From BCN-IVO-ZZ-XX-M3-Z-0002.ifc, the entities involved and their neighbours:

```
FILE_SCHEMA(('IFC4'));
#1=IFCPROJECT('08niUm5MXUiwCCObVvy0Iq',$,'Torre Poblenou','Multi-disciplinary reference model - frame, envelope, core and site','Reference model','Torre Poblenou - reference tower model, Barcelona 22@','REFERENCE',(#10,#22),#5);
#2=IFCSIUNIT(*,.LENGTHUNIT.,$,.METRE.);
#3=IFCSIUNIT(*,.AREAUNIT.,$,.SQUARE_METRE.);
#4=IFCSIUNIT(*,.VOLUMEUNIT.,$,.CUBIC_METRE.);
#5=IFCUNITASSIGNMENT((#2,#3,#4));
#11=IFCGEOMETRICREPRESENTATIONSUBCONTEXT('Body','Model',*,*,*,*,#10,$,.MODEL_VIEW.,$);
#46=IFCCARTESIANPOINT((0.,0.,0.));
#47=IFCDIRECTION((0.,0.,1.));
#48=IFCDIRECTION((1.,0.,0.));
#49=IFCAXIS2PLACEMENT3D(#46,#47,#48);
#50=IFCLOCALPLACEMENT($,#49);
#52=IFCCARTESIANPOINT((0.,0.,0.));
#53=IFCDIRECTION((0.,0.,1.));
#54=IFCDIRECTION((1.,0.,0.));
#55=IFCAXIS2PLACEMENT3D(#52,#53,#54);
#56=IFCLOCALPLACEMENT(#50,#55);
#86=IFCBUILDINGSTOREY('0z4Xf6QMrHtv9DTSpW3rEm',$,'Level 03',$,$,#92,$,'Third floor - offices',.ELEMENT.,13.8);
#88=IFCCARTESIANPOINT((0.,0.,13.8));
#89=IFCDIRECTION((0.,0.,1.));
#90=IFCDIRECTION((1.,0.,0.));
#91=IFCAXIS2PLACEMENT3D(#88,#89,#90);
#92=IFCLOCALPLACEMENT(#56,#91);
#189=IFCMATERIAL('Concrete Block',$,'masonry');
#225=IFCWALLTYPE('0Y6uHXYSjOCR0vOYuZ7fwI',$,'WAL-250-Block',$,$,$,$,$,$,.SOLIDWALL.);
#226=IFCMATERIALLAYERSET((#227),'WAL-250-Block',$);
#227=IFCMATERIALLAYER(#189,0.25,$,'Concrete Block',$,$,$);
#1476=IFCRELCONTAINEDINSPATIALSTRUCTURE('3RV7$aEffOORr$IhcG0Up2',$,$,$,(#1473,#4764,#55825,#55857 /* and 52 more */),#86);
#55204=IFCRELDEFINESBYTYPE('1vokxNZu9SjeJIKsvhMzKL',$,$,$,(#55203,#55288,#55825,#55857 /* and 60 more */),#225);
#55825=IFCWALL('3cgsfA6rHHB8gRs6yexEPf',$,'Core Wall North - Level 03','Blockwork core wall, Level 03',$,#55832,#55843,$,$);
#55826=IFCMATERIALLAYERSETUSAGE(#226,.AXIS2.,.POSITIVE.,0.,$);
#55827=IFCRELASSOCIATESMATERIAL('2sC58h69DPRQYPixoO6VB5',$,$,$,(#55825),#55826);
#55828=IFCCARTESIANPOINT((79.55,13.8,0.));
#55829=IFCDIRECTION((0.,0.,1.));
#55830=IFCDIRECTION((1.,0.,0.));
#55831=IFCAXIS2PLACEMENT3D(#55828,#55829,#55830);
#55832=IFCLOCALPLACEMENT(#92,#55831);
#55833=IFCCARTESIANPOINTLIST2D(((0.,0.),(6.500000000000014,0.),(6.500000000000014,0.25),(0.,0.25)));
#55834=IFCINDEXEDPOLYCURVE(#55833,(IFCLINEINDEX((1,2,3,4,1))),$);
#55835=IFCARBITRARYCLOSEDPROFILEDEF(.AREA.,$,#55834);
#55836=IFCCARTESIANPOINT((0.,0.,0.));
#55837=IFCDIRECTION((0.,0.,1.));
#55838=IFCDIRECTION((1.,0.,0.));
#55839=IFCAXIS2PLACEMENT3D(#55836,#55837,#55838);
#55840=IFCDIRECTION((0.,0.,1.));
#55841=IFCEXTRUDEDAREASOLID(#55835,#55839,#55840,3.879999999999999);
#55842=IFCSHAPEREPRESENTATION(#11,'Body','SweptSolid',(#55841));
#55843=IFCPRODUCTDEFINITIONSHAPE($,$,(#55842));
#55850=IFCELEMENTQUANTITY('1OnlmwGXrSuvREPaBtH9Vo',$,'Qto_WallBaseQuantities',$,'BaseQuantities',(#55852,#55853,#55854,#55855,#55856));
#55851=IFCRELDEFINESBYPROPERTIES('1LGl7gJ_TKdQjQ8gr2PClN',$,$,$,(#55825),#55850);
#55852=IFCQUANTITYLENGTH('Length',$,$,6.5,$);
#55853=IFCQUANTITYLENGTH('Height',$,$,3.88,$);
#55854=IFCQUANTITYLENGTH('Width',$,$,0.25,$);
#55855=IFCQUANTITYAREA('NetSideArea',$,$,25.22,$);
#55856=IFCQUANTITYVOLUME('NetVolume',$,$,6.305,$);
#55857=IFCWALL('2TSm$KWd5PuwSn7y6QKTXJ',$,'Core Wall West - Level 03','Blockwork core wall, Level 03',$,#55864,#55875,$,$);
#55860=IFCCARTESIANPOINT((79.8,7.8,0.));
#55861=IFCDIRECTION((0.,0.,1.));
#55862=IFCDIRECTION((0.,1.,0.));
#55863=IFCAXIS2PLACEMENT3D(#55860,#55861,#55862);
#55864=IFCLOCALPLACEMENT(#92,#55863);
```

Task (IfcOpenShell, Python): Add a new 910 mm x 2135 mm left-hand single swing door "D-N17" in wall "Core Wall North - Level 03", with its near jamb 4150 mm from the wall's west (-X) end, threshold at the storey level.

```python
import numpy as np
import ifcopenshell
import ifcopenshell.api.feature
import ifcopenshell.api.geometry
import ifcopenshell.api.pset
import ifcopenshell.api.root
import ifcopenshell.api.spatial
import ifcopenshell.geom
import ifcopenshell.util.element
import ifcopenshell.util.placement
import ifcopenshell.util.representation
import ifcopenshell.util.shape
import ifcopenshell.util.unit

model = ifcopenshell.open("BCN-IVO-ZZ-XX-M3-Z-0002.ifc")
unit_scale = ifcopenshell.util.unit.calculate_unit_scale(model)
area_scale = ifcopenshell.util.unit.calculate_unit_scale(model, "AREAUNIT")
volume_scale = ifcopenshell.util.unit.calculate_unit_scale(model, "VOLUMEUNIT")
settings = ifcopenshell.geom.settings()


def volume(element):
    """Net volume in cubic metres, openings subtracted."""
    shape = ifcopenshell.geom.create_shape(settings, element)
    return ifcopenshell.util.shape.get_volume(shape.geometry)


wall = model.by_guid("3cgsfA6rHHB8gRs6yexEPf")
storey = ifcopenshell.util.element.get_container(wall, ifc_class="IfcBuildingStorey")
context = ifcopenshell.util.representation.get_context(model, "Model", "Body", "MODEL_VIEW")
before = volume(wall)

width, height, from_end, sill = 0.91, 2.135, 4.15, 0.0  # metres

# The wall runs along its own X axis, and the end named is its -X end.
wall_shape = ifcopenshell.geom.create_shape(settings, wall)
x, y, z = ifcopenshell.util.shape.get_vertices(wall_shape.geometry).T
start = x.min() + from_end
face, thickness = float(y.min()), float(y.max() - y.min())
wall_matrix = ifcopenshell.util.placement.get_local_placement(wall.ObjectPlacement)
level = ifcopenshell.util.placement.get_local_placement(storey.ObjectPlacement)[2, 3]


def in_wall(x, y):
    """Placement at x, y metres in the wall's axes, at sill height."""
    matrix = wall_matrix.copy()
    matrix[:, 3] = wall_matrix @ np.array([x / unit_scale, y / unit_scale, 0.0, 1.0])
    matrix[2, 3] = level + sill / unit_scale
    return matrix


# Opening: a box that overshoots both wall faces by 50 mm.
opening = ifcopenshell.api.root.create_entity(model, ifc_class="IfcOpeningElement", predefined_type="OPENING")
box = ifcopenshell.api.geometry.add_wall_representation(
    model, context=context, length=width, height=height, thickness=thickness + 0.1
)
ifcopenshell.api.geometry.assign_representation(model, product=opening, representation=box)
ifcopenshell.api.geometry.edit_object_placement(model, product=opening, matrix=in_wall(start, face - 0.05), is_si=False)
ifcopenshell.api.feature.add_feature(model, feature=opening, element=wall)

door = ifcopenshell.api.root.create_entity(model, ifc_class="IfcDoor", name="D-N17", predefined_type="DOOR")
door.OverallWidth, door.OverallHeight = width / unit_scale, height / unit_scale
door.OperationType = "SINGLE_SWING_LEFT"
body = ifcopenshell.api.geometry.add_door_representation(
    model,
    context=context,
    overall_width=door.OverallWidth,
    overall_height=door.OverallHeight,
    operation_type="SINGLE_SWING_LEFT",
    lining_properties={"LiningDepth": thickness / unit_scale, "ThresholdDepth": thickness / unit_scale},
)
ifcopenshell.api.geometry.assign_representation(model, product=door, representation=body)
ifcopenshell.api.spatial.assign_container(model, products=[door], relating_structure=storey)
ifcopenshell.api.feature.add_filling(model, opening=opening, element=door)

# The lining spans the wall, so the door starts at the wall face.
ifcopenshell.api.geometry.edit_object_placement(model, product=door, matrix=in_wall(start, face), is_si=False)

after = volume(wall)

# Update the wall's stored quantities.
qto = model.by_id(ifcopenshell.util.element.get_pset(wall, "Qto_WallBaseQuantities", should_inherit=False)["id"])
ifcopenshell.api.pset.edit_qto(model, qto=qto, properties={
    "NetSideArea": after / thickness / area_scale,
    "NetVolume": after / volume_scale,
})

print(f"wall volume {before:.3f} -> {after:.3f} m3")

model.write("BCN-IVO-ZZ-XX-M3-Z-0002-out.ifc")
```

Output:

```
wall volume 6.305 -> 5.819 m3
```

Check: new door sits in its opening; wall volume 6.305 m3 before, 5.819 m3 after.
